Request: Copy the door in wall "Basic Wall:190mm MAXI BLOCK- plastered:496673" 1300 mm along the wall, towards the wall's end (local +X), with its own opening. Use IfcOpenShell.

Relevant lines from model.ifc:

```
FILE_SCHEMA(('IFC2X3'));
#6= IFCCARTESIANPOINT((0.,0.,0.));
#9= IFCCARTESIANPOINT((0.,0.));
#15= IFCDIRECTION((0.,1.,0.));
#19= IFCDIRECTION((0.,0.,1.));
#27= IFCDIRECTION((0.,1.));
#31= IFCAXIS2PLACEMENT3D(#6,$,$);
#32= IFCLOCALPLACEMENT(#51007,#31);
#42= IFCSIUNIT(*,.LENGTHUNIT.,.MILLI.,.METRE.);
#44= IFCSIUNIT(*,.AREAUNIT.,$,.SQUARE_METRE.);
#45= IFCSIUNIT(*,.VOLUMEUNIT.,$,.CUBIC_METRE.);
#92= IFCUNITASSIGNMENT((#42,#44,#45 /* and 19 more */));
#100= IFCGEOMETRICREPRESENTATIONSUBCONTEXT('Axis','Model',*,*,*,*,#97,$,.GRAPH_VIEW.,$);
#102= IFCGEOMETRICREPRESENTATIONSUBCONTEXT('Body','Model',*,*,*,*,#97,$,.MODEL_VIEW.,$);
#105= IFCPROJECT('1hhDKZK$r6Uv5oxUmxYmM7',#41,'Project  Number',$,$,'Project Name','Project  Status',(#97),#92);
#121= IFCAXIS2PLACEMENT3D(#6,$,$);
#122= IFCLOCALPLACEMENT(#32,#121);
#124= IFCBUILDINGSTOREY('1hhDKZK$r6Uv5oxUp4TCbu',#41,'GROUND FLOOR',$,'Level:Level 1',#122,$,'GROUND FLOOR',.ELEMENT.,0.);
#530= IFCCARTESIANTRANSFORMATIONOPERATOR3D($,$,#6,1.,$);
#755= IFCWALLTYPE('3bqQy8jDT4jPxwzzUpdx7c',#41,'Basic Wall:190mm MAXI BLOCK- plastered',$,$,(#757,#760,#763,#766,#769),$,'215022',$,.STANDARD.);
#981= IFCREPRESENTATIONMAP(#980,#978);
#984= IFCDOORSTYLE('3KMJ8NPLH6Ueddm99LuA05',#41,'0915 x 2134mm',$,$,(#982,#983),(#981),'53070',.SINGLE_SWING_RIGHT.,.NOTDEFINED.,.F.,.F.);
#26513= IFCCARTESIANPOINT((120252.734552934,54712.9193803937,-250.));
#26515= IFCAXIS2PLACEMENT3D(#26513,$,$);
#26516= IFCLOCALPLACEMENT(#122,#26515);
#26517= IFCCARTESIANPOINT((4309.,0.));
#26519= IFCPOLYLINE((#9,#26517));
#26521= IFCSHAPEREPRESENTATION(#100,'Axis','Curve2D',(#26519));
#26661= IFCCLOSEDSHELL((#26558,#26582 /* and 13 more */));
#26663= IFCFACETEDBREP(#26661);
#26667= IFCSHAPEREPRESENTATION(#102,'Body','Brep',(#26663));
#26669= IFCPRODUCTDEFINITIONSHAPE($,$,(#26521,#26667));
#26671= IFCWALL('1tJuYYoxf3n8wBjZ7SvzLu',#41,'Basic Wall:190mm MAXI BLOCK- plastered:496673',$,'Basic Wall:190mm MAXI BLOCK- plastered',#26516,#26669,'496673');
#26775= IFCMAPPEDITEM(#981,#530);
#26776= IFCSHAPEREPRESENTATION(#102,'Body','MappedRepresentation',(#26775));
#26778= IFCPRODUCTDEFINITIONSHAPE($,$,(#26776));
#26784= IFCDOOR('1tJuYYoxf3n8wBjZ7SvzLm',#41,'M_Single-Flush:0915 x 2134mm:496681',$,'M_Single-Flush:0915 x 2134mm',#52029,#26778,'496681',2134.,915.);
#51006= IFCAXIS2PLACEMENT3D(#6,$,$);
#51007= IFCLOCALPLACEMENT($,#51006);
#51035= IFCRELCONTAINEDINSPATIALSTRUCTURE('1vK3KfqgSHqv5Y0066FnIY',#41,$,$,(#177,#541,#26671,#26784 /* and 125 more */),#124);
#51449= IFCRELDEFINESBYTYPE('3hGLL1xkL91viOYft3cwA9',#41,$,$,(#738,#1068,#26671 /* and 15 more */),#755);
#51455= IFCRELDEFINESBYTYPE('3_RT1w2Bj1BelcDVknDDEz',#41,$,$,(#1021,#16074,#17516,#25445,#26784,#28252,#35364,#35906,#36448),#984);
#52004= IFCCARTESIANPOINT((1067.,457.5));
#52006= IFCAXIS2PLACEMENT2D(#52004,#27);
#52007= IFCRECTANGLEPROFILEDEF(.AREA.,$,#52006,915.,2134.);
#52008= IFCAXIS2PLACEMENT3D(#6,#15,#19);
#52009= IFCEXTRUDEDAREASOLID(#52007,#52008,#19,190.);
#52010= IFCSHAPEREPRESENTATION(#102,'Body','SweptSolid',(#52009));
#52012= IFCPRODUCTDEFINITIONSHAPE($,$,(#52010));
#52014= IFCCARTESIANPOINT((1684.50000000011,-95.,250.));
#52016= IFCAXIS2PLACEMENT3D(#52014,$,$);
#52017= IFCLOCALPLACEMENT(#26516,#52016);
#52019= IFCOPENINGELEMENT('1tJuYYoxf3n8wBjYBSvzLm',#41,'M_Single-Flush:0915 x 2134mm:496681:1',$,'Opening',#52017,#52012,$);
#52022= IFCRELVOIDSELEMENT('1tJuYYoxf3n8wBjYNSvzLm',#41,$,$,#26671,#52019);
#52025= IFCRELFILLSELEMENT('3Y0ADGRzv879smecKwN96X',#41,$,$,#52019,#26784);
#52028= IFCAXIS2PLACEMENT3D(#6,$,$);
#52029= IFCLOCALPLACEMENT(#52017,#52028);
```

```python
import ifcopenshell
import ifcopenshell.api.feature
import ifcopenshell.api.geometry
import ifcopenshell.api.root
import ifcopenshell.geom
import ifcopenshell.util.element
import ifcopenshell.util.placement
import ifcopenshell.util.shape

model = ifcopenshell.open("model.ifc")
settings = ifcopenshell.geom.settings()


def volume(element):
    """Net volume in cubic metres, openings subtracted."""
    shape = ifcopenshell.geom.create_shape(settings, element)
    return ifcopenshell.util.shape.get_volume(shape.geometry)


def reuse_history(source, copy):
    """copy_class also copies each property set's owner history, people and application; keep the originals."""
    for rel in copy.IsDefinedBy:
        if rel.is_a("IfcRelDefinesByProperties") and (history := rel.RelatingPropertyDefinition.OwnerHistory):
            rel.RelatingPropertyDefinition.OwnerHistory = source.OwnerHistory
            ifcopenshell.util.element.remove_deep2(model, history)


door = model.by_guid("1tJuYYoxf3n8wBjZ7SvzLm")
opening = door.FillsVoids[0].RelatingOpeningElement
wall = opening.VoidsElements[0].RelatingBuildingElement
before = volume(wall)
shift = ifcopenshell.util.placement.get_local_placement(wall.ObjectPlacement)[:3, 0] * 1300.0

# copy_class copies the void relationship, type, container and properties, but no geometry.
new_opening = ifcopenshell.api.root.copy_class(model, product=opening)
new_opening.Representation = ifcopenshell.util.element.copy_deep(
    model, opening.Representation, exclude=["IfcGeometricRepresentationContext", "IfcRepresentationMap"]
)
new_opening.Name = "M_Single-Flush:0915 x 2134mm"
new_door = ifcopenshell.api.root.copy_class(model, product=door)
new_door.Representation = ifcopenshell.util.element.copy_deep(
    model, door.Representation, exclude=["IfcGeometricRepresentationContext", "IfcRepresentationMap"]
)
new_door.Name = "M_Single-Flush:0915 x 2134mm"
new_door.Tag = None
reuse_history(door, new_door)
fills = ifcopenshell.api.feature.add_filling(model, opening=new_opening, element=new_door)
fills.OwnerHistory = new_door.OwnerHistory  # required in IFC2X3

for old, new in ((opening, new_opening), (door, new_door)):
    matrix = ifcopenshell.util.placement.get_local_placement(old.ObjectPlacement)
    matrix[:3, 3] += shift
    ifcopenshell.api.geometry.edit_object_placement(model, product=new, matrix=matrix, is_si=False)

after = volume(wall)

print(f"wall volume {before:.3f} -> {after:.3f} m3")

model.write("model_rev.ifc")
```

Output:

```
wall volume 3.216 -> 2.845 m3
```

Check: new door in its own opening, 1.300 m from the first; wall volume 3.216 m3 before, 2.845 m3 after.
